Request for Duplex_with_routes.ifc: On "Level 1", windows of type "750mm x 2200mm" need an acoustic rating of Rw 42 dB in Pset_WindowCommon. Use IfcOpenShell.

First a look at what the model holds.

```python
import ifcopenshell
import ifcopenshell.util.element

model = ifcopenshell.open("Duplex_with_routes.ifc")
print(model.schema)
storey = next(s for s in model.by_type("IfcBuildingStorey") if s.Name == "Level 1")
windows = [e for e in ifcopenshell.util.element.get_decomposition(storey) if e.is_a("IfcWindow")]
seen = {}
for e in windows:
    element_type = ifcopenshell.util.element.get_type(e)
    key = (element_type.Name if element_type != e and element_type else None, ifcopenshell.util.element.get_pset(e, "Pset_WindowCommon", "AcousticRating"))
    seen[key] = seen.get(key, 0) + 1
for (name, value), count in sorted(seen.items(), key=str):
    print(count, "x", name, "|", value)
```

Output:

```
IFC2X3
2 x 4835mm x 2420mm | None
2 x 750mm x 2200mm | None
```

```python
import ifcopenshell
import ifcopenshell.api.pset
import ifcopenshell.util.element

model = ifcopenshell.open("Duplex_with_routes.ifc")

storey = next(s for s in model.by_type("IfcBuildingStorey") if s.Name == "Level 1")
windows = [e for e in ifcopenshell.util.element.get_decomposition(storey) if e.is_a("IfcWindow")]

count = 0
for e in windows:
    element_type = ifcopenshell.util.element.get_type(e)
    if element_type in (None, e) or element_type.Name != "750mm x 2200mm":
        continue
    # add_pset returns the element's existing set when there is one.
    pset = ifcopenshell.api.pset.add_pset(model, product=e, name="Pset_WindowCommon")
    ifcopenshell.api.pset.edit_pset(model, pset=pset, properties={"AcousticRating": "Rw 42 dB"})
    count += 1

print(count, "windows updated")

model.write("Duplex_with_routes_updated.ifc")
```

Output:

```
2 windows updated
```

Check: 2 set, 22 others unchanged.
